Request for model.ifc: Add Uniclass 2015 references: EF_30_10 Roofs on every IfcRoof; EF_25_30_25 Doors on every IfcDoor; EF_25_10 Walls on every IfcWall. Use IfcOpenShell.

First a look at what the model holds.

```python
import ifcopenshell

model = ifcopenshell.open("model.ifc")
print(model.schema)
print("classifications:", [c.Name for c in model.by_type("IfcClassification")])
for ifc_class in ("IfcDoor", "IfcRoof", "IfcStair", "IfcWall", "IfcWindow"):
    print(ifc_class, len(model.by_type(ifc_class)))
```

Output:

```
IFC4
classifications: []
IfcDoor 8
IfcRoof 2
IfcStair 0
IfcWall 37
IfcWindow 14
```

```python
import ifcopenshell
import ifcopenshell.api.classification

model = ifcopenshell.open("model.ifc")

system = ifcopenshell.api.classification.add_classification(model, classification="Uniclass 2015")

codes = {
    "IfcRoof": ("EF_30_10", "Roofs"),
    "IfcDoor": ("EF_25_30_25", "Doors"),
    "IfcWall": ("EF_25_10", "Walls"),
}
for ifc_class, (code, name) in codes.items():
    products = model.by_type(ifc_class)
    ifcopenshell.api.classification.add_reference(
        model, products=products, classification=system, identification=code, name=name
    )
    print(code, len(products))

model.write("model_edited.ifc")
```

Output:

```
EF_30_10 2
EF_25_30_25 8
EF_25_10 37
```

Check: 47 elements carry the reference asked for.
